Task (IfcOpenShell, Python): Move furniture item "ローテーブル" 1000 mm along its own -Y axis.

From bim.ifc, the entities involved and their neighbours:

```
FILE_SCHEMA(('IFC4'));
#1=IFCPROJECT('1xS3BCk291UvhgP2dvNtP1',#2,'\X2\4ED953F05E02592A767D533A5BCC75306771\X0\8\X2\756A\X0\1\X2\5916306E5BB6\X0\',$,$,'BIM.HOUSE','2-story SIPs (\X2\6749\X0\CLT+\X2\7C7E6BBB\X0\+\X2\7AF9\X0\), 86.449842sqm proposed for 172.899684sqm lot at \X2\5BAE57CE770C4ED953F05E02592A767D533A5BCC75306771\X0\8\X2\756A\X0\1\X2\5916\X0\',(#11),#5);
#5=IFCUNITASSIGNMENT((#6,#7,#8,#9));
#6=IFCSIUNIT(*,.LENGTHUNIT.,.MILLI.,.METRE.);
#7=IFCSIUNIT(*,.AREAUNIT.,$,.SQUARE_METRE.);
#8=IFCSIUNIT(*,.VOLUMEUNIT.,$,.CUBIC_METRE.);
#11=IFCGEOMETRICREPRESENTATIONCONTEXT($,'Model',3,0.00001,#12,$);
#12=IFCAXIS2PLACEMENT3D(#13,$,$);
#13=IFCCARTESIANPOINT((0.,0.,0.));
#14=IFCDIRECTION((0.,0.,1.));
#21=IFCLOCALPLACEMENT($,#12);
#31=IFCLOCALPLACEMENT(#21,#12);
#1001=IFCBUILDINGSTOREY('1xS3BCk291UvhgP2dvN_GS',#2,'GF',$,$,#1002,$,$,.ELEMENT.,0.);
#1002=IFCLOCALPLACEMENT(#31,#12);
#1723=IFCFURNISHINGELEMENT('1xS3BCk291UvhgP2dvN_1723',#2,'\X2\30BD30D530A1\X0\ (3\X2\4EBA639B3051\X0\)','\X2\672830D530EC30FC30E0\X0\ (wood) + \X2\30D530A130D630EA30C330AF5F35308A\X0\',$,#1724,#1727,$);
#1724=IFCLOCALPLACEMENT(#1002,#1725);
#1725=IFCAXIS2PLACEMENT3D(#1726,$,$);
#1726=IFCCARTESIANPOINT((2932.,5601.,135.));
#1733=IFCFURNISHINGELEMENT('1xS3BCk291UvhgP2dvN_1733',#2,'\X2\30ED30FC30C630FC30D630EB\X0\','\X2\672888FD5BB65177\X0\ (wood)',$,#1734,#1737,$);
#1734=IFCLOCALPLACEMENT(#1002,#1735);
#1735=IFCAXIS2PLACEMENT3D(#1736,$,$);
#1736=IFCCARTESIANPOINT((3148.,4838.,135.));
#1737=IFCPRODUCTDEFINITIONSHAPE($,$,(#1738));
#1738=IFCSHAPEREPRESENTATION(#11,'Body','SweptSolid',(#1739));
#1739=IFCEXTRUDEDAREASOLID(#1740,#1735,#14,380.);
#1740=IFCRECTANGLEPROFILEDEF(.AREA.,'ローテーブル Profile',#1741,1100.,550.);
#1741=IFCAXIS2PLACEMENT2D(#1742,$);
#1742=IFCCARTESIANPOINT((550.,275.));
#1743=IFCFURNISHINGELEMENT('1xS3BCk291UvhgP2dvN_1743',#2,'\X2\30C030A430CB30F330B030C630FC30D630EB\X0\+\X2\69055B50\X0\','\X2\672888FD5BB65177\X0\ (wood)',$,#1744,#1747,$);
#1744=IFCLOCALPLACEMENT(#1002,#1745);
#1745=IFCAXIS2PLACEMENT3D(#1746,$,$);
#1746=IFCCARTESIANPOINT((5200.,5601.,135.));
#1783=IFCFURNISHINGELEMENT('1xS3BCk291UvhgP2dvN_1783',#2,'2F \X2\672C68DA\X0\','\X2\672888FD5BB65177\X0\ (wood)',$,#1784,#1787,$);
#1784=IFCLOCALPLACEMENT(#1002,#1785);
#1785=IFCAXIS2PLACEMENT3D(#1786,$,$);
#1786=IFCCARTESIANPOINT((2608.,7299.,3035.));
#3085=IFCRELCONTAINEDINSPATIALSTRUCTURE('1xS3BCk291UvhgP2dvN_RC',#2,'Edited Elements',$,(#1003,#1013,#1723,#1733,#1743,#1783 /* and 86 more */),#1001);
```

```python
import ifcopenshell
import ifcopenshell.api.geometry
import ifcopenshell.util.placement

model = ifcopenshell.open("bim.ifc")

item = model.by_guid("1xS3BCk291UvhgP2dvN_1733")
matrix = ifcopenshell.util.placement.get_local_placement(item.ObjectPlacement)
matrix[:3, 3] -= matrix[:3, 1] * 1000.0
ifcopenshell.api.geometry.edit_object_placement(model, product=item, matrix=matrix, is_si=False)

print(ifcopenshell.util.placement.get_local_placement(item.ObjectPlacement).round(3) + 0.0)

model.write("bim_edited.ifc")
```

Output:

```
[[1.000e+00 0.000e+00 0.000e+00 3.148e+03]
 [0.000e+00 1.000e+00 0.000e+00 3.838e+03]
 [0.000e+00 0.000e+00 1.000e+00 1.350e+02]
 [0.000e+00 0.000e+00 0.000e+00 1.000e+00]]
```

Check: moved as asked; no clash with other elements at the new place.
